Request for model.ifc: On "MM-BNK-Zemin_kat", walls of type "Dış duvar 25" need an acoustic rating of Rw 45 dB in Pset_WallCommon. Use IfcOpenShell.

First a look at what the model holds.

```python
import ifcopenshell
import ifcopenshell.util.element

model = ifcopenshell.open("model.ifc")
print(model.schema)
storey = next(s for s in model.by_type("IfcBuildingStorey") if s.Name == "MM-BNK-Zemin_kat")
walls = [e for e in ifcopenshell.util.element.get_decomposition(storey) if e.is_a("IfcWall")]
seen = {}
for e in walls:
    element_type = ifcopenshell.util.element.get_type(e)
    key = (element_type.Name if element_type != e and element_type else None, ifcopenshell.util.element.get_pset(e, "Pset_WallCommon", "AcousticRating"))
    seen[key] = seen.get(key, 0) + 1
for (name, value), count in sorted(seen.items(), key=str):
    print(count, "x", name, "|", value)
```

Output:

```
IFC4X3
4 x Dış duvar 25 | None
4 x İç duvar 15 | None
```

```python
import ifcopenshell
import ifcopenshell.api.pset
import ifcopenshell.util.element

model = ifcopenshell.open("model.ifc")

storey = next(s for s in model.by_type("IfcBuildingStorey") if s.Name == "MM-BNK-Zemin_kat")
walls = [e for e in ifcopenshell.util.element.get_decomposition(storey) if e.is_a("IfcWall")]

count = 0
for e in walls:
    element_type = ifcopenshell.util.element.get_type(e)
    if element_type in (None, e) or element_type.Name != "Dış duvar 25":
        continue
    # add_pset returns the element's existing set when there is one.
    pset = ifcopenshell.api.pset.add_pset(model, product=e, name="Pset_WallCommon")
    ifcopenshell.api.pset.edit_pset(model, pset=pset, properties={"AcousticRating": "Rw 45 dB"})
    count += 1

print(count, "walls updated")

model.write("model_v2.ifc")
```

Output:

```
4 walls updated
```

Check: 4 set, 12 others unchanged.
